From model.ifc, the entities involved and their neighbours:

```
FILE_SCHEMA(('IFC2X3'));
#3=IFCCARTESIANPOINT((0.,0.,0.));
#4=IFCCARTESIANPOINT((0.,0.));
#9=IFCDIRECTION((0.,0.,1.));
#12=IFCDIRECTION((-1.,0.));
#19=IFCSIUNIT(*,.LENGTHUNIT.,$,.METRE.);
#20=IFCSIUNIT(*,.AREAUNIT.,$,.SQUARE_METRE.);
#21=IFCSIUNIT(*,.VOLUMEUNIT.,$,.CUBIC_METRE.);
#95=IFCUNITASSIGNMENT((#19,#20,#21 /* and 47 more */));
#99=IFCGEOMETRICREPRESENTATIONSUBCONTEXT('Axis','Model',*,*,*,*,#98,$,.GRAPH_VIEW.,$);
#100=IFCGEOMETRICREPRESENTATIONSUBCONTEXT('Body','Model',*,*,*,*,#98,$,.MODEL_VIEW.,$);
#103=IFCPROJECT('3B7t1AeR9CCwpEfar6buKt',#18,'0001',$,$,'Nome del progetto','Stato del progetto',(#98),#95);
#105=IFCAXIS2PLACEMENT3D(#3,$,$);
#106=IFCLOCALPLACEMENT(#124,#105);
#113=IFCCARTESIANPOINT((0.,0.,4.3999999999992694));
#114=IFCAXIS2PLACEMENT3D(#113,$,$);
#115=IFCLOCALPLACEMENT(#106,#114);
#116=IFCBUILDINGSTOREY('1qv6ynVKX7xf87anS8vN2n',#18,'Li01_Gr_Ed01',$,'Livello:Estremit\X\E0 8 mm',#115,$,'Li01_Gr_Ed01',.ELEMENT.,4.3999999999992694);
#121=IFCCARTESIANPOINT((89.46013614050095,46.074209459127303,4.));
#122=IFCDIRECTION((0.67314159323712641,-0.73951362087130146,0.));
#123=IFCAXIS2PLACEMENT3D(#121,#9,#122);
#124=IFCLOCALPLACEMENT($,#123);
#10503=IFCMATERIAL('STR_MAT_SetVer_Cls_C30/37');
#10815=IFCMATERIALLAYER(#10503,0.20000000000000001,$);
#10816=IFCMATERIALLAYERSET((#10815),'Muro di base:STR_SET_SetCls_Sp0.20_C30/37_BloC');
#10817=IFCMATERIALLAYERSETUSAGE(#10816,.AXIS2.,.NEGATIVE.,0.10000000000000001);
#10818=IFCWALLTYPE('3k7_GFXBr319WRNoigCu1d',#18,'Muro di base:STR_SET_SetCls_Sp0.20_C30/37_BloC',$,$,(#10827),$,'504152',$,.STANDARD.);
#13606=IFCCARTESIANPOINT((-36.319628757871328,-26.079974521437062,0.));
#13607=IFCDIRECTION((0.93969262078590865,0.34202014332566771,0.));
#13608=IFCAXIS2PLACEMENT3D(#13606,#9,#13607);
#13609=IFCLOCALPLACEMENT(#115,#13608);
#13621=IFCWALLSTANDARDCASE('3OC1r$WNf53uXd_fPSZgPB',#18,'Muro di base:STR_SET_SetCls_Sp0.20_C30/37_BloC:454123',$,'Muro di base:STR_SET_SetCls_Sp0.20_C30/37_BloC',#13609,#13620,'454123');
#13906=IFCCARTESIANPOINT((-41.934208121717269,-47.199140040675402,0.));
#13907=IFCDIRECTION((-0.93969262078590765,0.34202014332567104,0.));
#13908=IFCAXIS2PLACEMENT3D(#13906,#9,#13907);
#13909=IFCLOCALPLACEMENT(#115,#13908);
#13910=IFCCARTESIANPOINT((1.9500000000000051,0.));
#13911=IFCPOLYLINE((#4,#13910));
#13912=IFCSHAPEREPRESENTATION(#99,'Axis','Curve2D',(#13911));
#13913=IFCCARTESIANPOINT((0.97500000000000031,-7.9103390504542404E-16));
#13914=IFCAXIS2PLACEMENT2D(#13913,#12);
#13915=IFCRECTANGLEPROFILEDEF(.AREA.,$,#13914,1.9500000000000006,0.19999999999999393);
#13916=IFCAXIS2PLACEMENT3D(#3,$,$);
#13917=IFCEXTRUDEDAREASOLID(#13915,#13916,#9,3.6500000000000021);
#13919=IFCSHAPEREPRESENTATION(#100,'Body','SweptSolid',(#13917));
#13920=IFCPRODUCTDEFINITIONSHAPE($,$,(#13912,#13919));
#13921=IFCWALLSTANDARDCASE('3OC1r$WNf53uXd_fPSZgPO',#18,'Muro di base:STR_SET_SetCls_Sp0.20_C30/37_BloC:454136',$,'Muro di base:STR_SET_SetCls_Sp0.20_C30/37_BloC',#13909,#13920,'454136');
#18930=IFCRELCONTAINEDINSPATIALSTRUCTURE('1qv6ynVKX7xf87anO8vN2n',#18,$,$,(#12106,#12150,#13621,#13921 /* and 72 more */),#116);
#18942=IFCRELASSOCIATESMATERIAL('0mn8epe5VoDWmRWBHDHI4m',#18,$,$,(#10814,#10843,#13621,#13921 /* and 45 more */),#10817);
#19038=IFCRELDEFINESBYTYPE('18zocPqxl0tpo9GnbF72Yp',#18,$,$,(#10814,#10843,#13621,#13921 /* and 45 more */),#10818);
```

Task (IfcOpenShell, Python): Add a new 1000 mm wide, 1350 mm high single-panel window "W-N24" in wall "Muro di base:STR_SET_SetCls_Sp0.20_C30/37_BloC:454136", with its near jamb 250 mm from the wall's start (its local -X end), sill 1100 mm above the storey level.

```python
import numpy as np
import ifcopenshell
import ifcopenshell.api.feature
import ifcopenshell.api.geometry
import ifcopenshell.api.root
import ifcopenshell.api.spatial
import ifcopenshell.api.type
import ifcopenshell.geom
import ifcopenshell.util.element
import ifcopenshell.util.placement
import ifcopenshell.util.representation
import ifcopenshell.util.shape
import ifcopenshell.util.unit

model = ifcopenshell.open("model.ifc")
unit_scale = ifcopenshell.util.unit.calculate_unit_scale(model)
settings = ifcopenshell.geom.settings()


def volume(element):
    """Net volume in cubic metres, openings subtracted."""
    shape = ifcopenshell.geom.create_shape(settings, element)
    return ifcopenshell.util.shape.get_volume(shape.geometry)


wall = model.by_guid("3OC1r$WNf53uXd_fPSZgPO")
storey = ifcopenshell.util.element.get_container(wall, ifc_class="IfcBuildingStorey")
context = ifcopenshell.util.representation.get_context(model, "Model", "Body", "MODEL_VIEW")
before = volume(wall)

width, height, from_end, sill = 1, 1.35, 0.25, 1.1  # metres

# The wall runs along its own X axis, and the end named is its -X end.
wall_shape = ifcopenshell.geom.create_shape(settings, wall)
x, y, z = ifcopenshell.util.shape.get_vertices(wall_shape.geometry).T
start = x.min() + from_end
face, thickness = float(y.min()), float(y.max() - y.min())
wall_matrix = ifcopenshell.util.placement.get_local_placement(wall.ObjectPlacement)
level = ifcopenshell.util.placement.get_local_placement(storey.ObjectPlacement)[2, 3]


def in_wall(x, y):
    """Placement at x, y metres in the wall's axes, at sill height."""
    matrix = wall_matrix.copy()
    matrix[:, 3] = wall_matrix @ np.array([x / unit_scale, y / unit_scale, 0.0, 1.0])
    matrix[2, 3] = level + sill / unit_scale
    return matrix


# Opening: a box that overshoots both wall faces by 50 mm.
opening = ifcopenshell.api.root.create_entity(model, ifc_class="IfcOpeningElement")
box = ifcopenshell.api.geometry.add_wall_representation(
    model, context=context, length=width, height=height, thickness=thickness + 0.1
)
ifcopenshell.api.geometry.assign_representation(model, product=opening, representation=box)
ifcopenshell.api.geometry.edit_object_placement(model, product=opening, matrix=in_wall(start, face - 0.05), is_si=False)
ifcopenshell.api.feature.add_feature(model, feature=opening, element=wall)

window = ifcopenshell.api.root.create_entity(model, ifc_class="IfcWindow", name="W-N24")
window.OverallWidth, window.OverallHeight = width / unit_scale, height / unit_scale
body = ifcopenshell.api.geometry.add_window_representation(
    model,
    context=context,
    overall_width=window.OverallWidth,
    overall_height=window.OverallHeight,
    partition_type="SINGLE_PANEL",
)
ifcopenshell.api.geometry.assign_representation(model, product=window, representation=body)
ifcopenshell.api.spatial.assign_container(model, products=[window], relating_structure=storey)
fills = ifcopenshell.api.feature.add_filling(model, opening=opening, element=window)
fills.OwnerHistory = window.OwnerHistory  # required in IFC2X3

# IFC2X3 keeps the operation on the window style.
style = ifcopenshell.api.root.create_entity(model, ifc_class="IfcWindowStyle", name="W-N24")
style.OperationType, style.ConstructionType = "SINGLE_PANEL", "NOTDEFINED"
style.ParameterTakesPrecedence = style.Sizeable = False
ifcopenshell.api.type.assign_type(model, related_objects=[window], relating_type=style)

# Centre the window in the wall's thickness.
ifcopenshell.api.geometry.edit_object_placement(model, product=window, matrix=in_wall(start, face), is_si=False)
window_shape = ifcopenshell.geom.create_shape(settings, window)
depth = ifcopenshell.util.shape.get_vertices(window_shape.geometry)[:, 1]
offset = face + thickness / 2 - (depth.min() + depth.max()) / 2
ifcopenshell.api.geometry.edit_object_placement(model, product=window, matrix=in_wall(start, offset), is_si=False)

after = volume(wall)

print(f"wall volume {before:.3f} -> {after:.3f} m3")

model.write("model-out.ifc")
```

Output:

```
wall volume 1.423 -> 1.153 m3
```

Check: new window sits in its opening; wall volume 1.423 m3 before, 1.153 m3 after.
